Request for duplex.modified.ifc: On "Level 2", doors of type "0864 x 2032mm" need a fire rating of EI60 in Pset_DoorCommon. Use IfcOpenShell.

First a look at what the model holds.

```python
import ifcopenshell
import ifcopenshell.util.element

model = ifcopenshell.open("duplex.modified.ifc")
print(model.schema)
storey = next(s for s in model.by_type("IfcBuildingStorey") if s.Name == "Level 2")
doors = [e for e in ifcopenshell.util.element.get_decomposition(storey) if e.is_a("IfcDoor")]
seen = {}
for e in doors:
    element_type = ifcopenshell.util.element.get_type(e)
    key = (element_type.Name if element_type != e and element_type else None, ifcopenshell.util.element.get_pset(e, "Pset_DoorCommon", "FireRating"))
    seen[key] = seen.get(key, 0) + 1
for (name, value), count in sorted(seen.items(), key=str):
    print(count, "x", name, "|", value)
```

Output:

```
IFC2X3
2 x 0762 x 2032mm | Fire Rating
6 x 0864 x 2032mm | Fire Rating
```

```python
import ifcopenshell
import ifcopenshell.api.pset
import ifcopenshell.util.element

model = ifcopenshell.open("duplex.modified.ifc")

storey = next(s for s in model.by_type("IfcBuildingStorey") if s.Name == "Level 2")
doors = [e for e in ifcopenshell.util.element.get_decomposition(storey) if e.is_a("IfcDoor")]

count = 0
for e in doors:
    element_type = ifcopenshell.util.element.get_type(e)
    if element_type in (None, e) or element_type.Name != "0864 x 2032mm":
        continue
    # add_pset returns the element's existing set when there is one.
    pset = ifcopenshell.api.pset.add_pset(model, product=e, name="Pset_DoorCommon")
    ifcopenshell.api.pset.edit_pset(model, pset=pset, properties={"FireRating": "EI60"})
    count += 1

print(count, "doors updated")

model.write("duplex.modified_rev.ifc")
```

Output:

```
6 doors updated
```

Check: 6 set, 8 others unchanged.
